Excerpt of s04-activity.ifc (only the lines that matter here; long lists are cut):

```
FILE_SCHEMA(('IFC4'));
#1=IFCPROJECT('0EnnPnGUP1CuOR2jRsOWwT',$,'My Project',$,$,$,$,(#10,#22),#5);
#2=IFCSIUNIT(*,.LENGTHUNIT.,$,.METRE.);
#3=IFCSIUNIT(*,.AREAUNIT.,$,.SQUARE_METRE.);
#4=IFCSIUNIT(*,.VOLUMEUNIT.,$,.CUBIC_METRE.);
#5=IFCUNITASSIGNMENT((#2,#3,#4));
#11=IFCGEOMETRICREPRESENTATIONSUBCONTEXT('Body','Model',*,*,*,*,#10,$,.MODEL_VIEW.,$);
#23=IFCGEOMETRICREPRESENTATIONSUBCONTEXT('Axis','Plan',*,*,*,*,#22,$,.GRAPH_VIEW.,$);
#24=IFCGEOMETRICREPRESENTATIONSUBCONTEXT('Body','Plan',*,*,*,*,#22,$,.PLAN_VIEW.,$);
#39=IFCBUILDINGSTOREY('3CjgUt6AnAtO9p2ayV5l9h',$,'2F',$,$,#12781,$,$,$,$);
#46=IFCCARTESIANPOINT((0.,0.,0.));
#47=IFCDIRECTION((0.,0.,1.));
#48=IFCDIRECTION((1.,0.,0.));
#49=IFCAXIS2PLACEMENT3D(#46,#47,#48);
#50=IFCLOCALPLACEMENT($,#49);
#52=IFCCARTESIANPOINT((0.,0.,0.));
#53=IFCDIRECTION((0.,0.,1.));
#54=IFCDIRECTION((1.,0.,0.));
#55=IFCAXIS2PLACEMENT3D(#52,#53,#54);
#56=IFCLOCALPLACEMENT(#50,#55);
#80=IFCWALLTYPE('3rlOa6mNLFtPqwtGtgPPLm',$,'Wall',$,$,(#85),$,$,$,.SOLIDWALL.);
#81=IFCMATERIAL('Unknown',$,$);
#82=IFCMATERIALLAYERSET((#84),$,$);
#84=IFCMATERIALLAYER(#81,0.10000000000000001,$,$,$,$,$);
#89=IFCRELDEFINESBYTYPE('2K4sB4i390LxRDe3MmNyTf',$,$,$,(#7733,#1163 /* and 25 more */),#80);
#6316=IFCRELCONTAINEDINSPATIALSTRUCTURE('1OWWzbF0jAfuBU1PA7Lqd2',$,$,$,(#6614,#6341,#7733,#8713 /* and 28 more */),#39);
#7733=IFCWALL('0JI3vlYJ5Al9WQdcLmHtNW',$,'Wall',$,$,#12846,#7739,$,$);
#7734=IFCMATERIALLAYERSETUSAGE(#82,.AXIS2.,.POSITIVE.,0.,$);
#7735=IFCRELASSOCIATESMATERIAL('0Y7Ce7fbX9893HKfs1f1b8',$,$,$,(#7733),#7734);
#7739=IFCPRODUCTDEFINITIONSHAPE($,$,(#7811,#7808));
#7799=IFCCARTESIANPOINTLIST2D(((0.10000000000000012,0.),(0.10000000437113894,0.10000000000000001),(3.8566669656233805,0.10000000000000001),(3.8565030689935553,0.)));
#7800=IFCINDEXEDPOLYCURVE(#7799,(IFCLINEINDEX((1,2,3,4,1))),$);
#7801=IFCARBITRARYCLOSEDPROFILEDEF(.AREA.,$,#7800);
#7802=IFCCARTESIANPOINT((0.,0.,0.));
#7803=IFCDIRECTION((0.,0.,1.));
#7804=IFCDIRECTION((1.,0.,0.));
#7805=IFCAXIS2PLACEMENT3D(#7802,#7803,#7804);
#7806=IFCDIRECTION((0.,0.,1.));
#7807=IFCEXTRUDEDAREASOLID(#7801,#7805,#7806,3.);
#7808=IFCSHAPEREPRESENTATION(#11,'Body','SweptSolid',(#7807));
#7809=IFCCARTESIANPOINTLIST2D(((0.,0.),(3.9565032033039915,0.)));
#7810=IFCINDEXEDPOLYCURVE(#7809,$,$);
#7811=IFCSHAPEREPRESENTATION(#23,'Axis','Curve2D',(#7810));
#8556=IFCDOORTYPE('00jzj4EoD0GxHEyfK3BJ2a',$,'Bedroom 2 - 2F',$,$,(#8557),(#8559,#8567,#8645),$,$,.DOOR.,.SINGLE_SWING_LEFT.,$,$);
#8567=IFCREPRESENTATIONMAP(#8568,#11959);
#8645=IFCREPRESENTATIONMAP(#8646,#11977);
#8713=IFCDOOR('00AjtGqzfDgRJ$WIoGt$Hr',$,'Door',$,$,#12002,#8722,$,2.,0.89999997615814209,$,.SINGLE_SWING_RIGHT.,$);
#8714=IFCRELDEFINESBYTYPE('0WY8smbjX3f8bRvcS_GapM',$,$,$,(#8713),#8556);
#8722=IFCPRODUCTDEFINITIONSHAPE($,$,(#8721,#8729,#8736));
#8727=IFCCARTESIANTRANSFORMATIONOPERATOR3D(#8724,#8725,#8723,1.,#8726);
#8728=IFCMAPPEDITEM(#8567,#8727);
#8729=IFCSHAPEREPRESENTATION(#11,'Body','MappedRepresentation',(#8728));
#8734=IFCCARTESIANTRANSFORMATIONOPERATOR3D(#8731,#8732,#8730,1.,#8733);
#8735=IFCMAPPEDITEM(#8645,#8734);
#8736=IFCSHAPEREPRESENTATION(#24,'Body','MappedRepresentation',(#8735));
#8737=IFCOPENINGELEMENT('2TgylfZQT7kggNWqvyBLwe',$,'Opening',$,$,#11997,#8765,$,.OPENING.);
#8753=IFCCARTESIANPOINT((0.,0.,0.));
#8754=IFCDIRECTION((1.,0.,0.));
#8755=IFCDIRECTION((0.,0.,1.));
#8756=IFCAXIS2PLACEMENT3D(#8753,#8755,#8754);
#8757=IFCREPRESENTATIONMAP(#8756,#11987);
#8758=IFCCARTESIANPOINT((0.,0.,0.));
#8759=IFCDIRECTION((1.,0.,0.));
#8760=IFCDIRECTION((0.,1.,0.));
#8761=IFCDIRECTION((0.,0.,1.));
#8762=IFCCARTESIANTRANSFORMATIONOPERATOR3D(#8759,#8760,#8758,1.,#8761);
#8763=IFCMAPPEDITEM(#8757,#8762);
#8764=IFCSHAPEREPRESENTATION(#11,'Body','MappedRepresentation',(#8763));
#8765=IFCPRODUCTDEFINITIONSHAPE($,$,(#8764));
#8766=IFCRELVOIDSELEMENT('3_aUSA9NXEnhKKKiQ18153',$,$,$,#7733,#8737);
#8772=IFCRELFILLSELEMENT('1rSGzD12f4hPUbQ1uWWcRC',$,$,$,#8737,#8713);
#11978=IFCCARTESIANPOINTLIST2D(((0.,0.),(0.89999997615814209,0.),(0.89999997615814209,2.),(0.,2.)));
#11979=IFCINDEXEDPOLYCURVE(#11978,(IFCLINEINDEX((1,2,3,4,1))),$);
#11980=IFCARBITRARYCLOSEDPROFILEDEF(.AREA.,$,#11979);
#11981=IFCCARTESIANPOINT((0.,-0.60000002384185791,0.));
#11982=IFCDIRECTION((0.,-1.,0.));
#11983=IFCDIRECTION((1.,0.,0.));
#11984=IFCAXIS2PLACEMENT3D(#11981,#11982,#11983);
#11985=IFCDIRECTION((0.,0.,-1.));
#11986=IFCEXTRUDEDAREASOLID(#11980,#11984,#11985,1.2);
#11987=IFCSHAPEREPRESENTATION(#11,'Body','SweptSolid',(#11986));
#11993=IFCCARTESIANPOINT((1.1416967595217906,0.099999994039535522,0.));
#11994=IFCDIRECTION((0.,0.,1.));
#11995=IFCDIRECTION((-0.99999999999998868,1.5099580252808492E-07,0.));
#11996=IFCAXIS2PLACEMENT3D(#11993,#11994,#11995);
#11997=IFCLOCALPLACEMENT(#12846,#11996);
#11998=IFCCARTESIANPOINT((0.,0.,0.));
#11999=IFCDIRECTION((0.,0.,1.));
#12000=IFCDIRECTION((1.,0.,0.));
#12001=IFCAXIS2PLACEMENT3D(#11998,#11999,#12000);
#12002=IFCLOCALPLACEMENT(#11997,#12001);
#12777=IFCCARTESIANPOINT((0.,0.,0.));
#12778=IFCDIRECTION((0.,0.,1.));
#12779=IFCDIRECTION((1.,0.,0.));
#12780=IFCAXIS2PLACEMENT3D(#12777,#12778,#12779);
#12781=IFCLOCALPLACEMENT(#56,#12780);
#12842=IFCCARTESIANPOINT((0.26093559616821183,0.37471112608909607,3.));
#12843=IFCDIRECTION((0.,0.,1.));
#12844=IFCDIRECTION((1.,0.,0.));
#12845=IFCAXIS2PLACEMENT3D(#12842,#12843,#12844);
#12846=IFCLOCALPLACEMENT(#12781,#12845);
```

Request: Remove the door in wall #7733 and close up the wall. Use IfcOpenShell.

```python
import ifcopenshell
import ifcopenshell.api.feature
import ifcopenshell.api.root
import ifcopenshell.geom
import ifcopenshell.util.shape

model = ifcopenshell.open("s04-activity.ifc")
settings = ifcopenshell.geom.settings()


def volume(element):
    """Net volume in cubic metres, openings subtracted."""
    shape = ifcopenshell.geom.create_shape(settings, element)
    return ifcopenshell.util.shape.get_volume(shape.geometry)


door = model.by_guid("00AjtGqzfDgRJ$WIoGt$Hr")
opening = door.FillsVoids[0].RelatingOpeningElement
wall = opening.VoidsElements[0].RelatingBuildingElement
before = volume(wall)

ifcopenshell.api.root.remove_product(model, product=door)
ifcopenshell.api.feature.remove_feature(model, feature=opening)

after = volume(wall)

print(f"wall volume {before:.3f} -> {after:.3f} m3")

model.write("s04-activity_rev.ifc")
```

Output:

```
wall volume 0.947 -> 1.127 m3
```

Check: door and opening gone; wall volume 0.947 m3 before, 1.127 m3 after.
